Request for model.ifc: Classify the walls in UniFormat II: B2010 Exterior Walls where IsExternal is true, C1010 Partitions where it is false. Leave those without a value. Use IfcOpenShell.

First a look at what the model holds.

```python
import ifcopenshell
import ifcopenshell.util.element

model = ifcopenshell.open("model.ifc")
print(model.schema)
print("classifications:", [c.Name for c in model.by_type("IfcClassification")])
values = [ifcopenshell.util.element.get_pset(e, "Pset_WallCommon", "IsExternal") for e in model.by_type("IfcWall")]
for value in (True, False, None):
    print("IsExternal", value, values.count(value))
```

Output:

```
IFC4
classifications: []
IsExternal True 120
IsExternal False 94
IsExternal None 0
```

```python
import ifcopenshell
import ifcopenshell.api.classification
import ifcopenshell.util.element

model = ifcopenshell.open("model.ifc")

system = ifcopenshell.api.classification.add_classification(model, classification="UniFormat II")

walls = model.by_type("IfcWall")
external = {e: ifcopenshell.util.element.get_pset(e, "Pset_WallCommon", "IsExternal") for e in walls}
for flag, code, name in ((True, "B2010", "Exterior Walls"), (False, "C1010", "Partitions")):
    products = [e for e in walls if external[e] is flag]
    ifcopenshell.api.classification.add_reference(
        model, products=products, classification=system, identification=code, name=name
    )
    print(code, len(products))

model.write("model_edited.ifc")
```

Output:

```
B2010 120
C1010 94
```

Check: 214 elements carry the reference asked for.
